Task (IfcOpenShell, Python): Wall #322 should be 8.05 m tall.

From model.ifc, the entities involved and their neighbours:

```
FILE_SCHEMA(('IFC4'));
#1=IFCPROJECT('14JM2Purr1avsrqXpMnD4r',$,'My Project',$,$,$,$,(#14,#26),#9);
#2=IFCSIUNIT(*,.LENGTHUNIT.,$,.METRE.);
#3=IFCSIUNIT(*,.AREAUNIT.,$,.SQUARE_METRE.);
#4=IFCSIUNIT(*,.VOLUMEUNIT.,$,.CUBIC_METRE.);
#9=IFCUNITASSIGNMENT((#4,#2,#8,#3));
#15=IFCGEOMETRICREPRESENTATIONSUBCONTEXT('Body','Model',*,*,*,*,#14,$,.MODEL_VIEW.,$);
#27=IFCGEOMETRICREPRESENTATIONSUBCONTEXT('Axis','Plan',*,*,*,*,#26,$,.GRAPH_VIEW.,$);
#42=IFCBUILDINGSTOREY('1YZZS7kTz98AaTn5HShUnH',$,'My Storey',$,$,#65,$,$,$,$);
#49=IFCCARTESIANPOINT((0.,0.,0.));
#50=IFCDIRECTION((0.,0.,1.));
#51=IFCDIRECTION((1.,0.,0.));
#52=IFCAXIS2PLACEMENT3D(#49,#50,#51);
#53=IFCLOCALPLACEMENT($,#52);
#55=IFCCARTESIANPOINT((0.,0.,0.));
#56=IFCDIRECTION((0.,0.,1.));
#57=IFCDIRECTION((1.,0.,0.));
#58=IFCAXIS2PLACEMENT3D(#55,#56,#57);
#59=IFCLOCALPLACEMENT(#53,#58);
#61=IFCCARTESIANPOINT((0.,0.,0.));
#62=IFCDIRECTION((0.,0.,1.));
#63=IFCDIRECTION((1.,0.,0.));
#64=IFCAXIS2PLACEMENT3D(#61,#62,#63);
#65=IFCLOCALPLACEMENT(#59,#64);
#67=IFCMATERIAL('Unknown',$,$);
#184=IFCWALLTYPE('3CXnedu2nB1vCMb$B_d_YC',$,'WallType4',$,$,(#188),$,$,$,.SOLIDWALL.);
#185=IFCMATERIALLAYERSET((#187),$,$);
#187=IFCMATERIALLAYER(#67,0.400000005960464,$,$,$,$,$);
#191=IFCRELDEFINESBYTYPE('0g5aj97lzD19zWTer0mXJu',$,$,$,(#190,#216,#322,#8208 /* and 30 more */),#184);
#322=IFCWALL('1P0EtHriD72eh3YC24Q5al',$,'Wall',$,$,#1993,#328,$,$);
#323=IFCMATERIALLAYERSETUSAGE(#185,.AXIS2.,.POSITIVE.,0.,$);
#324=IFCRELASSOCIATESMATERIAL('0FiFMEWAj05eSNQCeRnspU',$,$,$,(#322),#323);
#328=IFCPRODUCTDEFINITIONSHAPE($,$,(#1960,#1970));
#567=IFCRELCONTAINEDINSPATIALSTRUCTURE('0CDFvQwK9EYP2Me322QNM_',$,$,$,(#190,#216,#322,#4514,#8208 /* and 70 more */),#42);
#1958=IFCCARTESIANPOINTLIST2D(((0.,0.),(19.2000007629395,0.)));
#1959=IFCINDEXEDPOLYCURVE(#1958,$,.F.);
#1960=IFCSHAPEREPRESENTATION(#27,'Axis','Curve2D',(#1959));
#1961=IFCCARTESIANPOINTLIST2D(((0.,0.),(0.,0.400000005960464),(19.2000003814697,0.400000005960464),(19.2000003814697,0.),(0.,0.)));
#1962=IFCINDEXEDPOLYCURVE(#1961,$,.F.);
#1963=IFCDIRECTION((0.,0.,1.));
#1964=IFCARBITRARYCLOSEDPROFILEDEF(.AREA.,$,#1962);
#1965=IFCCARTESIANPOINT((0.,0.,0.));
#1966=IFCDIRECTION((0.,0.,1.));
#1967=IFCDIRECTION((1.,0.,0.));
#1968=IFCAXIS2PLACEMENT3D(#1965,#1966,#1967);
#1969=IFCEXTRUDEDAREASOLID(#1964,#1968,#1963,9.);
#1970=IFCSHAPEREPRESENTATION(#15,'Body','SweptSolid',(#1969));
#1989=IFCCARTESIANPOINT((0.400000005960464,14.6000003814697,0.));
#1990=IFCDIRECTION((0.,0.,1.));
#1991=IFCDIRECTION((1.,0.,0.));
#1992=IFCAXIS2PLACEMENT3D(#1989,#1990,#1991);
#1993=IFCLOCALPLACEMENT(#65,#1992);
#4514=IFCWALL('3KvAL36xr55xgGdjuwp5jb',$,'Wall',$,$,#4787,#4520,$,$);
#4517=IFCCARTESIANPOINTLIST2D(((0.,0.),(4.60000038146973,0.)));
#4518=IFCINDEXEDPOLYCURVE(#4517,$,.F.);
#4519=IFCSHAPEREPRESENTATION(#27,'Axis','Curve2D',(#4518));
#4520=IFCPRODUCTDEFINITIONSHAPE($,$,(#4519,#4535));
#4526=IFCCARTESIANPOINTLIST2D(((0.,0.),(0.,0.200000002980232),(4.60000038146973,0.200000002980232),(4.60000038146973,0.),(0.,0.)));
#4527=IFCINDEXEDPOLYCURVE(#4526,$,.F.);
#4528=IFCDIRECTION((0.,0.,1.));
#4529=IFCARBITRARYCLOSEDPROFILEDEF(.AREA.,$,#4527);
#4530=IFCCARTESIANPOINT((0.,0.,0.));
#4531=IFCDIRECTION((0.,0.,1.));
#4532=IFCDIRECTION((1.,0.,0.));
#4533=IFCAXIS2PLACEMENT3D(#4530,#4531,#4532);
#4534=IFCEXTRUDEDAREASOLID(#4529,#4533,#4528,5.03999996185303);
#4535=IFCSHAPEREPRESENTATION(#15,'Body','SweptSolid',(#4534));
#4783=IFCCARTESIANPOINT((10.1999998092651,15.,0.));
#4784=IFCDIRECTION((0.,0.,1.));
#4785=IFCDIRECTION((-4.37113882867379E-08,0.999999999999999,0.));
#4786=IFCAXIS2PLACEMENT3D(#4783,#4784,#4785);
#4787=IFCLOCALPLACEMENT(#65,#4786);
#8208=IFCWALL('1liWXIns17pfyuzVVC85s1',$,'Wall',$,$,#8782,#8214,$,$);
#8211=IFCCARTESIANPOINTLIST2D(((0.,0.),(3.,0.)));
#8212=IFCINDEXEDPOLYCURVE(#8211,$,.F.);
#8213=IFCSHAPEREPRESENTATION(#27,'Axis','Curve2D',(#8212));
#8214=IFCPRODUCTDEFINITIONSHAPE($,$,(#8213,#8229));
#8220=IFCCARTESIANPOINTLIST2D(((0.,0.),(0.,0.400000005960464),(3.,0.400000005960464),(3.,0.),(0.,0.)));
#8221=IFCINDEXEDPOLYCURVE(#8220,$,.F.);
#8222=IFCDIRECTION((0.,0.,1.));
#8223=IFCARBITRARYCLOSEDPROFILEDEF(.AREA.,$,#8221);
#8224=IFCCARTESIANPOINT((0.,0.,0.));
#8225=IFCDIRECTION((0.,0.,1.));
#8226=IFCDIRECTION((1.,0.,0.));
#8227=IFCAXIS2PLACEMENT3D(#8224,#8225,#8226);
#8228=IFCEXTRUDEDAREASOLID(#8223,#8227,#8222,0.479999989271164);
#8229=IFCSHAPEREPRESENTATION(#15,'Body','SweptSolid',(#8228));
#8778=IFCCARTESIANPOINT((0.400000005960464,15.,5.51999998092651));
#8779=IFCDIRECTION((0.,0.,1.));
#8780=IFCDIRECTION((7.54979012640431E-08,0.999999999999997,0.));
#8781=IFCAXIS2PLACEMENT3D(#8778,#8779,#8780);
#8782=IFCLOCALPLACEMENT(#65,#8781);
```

```python
import ifcopenshell
import ifcopenshell.geom
import ifcopenshell.util.representation
import ifcopenshell.util.shape
import ifcopenshell.util.unit

model = ifcopenshell.open("model.ifc")
unit_scale = ifcopenshell.util.unit.calculate_unit_scale(model)
settings = ifcopenshell.geom.settings()


def volume(element):
    """Net volume in cubic metres, openings subtracted."""
    shape = ifcopenshell.geom.create_shape(settings, element)
    return ifcopenshell.util.shape.get_volume(shape.geometry)


wall = model.by_guid("1P0EtHriD72eh3YC24Q5al")
before = volume(wall)

body = ifcopenshell.util.representation.get_representation(wall, "Model", "Body")
solid = body.Items[0]
old_height = solid.Depth
solid.Depth = 8.05 / unit_scale
after = volume(wall)

print(f"height {old_height:g} -> {solid.Depth:g}, volume {before:.3f} -> {after:.3f} m3")

model.write("model-out.ifc")
```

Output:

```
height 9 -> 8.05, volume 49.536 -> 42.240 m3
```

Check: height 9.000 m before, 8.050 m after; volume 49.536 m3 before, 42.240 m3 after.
